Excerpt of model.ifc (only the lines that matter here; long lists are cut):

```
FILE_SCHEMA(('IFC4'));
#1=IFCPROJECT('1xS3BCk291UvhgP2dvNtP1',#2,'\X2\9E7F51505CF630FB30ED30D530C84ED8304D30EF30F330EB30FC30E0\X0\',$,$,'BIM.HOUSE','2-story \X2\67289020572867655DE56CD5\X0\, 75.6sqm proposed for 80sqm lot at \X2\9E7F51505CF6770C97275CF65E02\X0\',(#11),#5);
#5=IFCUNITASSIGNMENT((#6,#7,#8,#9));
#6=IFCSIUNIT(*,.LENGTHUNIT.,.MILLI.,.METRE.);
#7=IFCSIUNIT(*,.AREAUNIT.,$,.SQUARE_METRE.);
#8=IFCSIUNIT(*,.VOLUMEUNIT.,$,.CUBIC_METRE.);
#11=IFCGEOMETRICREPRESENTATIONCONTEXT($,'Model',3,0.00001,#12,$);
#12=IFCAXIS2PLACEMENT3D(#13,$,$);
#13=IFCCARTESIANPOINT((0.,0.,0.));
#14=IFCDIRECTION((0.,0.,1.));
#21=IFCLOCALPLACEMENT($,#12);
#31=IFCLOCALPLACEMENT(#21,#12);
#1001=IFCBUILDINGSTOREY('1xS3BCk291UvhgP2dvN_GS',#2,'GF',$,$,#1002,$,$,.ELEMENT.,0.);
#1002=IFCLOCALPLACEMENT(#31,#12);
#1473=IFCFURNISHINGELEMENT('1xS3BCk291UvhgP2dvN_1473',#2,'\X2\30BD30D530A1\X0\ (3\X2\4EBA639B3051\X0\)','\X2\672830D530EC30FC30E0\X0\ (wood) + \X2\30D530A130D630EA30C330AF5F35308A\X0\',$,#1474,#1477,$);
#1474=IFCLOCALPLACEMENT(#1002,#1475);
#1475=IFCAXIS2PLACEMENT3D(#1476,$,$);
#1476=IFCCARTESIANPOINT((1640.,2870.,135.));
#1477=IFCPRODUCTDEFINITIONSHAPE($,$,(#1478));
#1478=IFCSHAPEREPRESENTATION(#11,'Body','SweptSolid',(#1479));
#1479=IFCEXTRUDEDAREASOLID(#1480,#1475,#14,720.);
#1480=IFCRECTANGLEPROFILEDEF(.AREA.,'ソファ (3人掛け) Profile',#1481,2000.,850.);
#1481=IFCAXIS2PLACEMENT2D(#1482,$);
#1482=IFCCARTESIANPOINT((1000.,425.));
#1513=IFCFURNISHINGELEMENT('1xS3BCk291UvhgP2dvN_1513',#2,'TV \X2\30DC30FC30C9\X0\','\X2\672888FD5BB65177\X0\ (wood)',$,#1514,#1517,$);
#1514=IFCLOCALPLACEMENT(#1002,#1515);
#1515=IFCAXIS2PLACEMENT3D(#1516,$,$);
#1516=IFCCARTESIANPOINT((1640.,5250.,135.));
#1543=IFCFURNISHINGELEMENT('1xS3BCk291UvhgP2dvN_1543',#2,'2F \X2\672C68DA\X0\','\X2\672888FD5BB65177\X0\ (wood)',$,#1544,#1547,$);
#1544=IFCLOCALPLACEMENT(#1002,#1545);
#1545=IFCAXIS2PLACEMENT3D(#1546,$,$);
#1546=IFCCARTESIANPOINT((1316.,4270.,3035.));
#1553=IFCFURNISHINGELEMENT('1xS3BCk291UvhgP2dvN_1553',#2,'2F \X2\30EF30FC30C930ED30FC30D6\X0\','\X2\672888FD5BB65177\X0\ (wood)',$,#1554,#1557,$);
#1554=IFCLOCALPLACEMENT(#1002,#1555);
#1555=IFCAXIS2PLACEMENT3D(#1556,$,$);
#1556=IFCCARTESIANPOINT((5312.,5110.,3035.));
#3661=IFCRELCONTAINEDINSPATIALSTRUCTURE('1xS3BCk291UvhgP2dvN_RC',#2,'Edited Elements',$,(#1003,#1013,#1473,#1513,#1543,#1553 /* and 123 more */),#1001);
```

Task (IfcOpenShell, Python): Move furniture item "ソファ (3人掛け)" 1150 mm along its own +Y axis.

```python
import ifcopenshell
import ifcopenshell.api.geometry
import ifcopenshell.util.placement

model = ifcopenshell.open("model.ifc")

item = model.by_id(1473)
matrix = ifcopenshell.util.placement.get_local_placement(item.ObjectPlacement)
matrix[:3, 3] += matrix[:3, 1] * 1150.0
ifcopenshell.api.geometry.edit_object_placement(model, product=item, matrix=matrix, is_si=False)

print(ifcopenshell.util.placement.get_local_placement(item.ObjectPlacement).round(3) + 0.0)

model.write("model_v2.ifc")
```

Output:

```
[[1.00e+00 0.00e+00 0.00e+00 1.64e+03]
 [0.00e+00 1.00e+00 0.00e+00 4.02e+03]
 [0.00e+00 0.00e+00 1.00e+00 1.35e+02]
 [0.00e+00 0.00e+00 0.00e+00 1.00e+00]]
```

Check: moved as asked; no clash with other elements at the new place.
